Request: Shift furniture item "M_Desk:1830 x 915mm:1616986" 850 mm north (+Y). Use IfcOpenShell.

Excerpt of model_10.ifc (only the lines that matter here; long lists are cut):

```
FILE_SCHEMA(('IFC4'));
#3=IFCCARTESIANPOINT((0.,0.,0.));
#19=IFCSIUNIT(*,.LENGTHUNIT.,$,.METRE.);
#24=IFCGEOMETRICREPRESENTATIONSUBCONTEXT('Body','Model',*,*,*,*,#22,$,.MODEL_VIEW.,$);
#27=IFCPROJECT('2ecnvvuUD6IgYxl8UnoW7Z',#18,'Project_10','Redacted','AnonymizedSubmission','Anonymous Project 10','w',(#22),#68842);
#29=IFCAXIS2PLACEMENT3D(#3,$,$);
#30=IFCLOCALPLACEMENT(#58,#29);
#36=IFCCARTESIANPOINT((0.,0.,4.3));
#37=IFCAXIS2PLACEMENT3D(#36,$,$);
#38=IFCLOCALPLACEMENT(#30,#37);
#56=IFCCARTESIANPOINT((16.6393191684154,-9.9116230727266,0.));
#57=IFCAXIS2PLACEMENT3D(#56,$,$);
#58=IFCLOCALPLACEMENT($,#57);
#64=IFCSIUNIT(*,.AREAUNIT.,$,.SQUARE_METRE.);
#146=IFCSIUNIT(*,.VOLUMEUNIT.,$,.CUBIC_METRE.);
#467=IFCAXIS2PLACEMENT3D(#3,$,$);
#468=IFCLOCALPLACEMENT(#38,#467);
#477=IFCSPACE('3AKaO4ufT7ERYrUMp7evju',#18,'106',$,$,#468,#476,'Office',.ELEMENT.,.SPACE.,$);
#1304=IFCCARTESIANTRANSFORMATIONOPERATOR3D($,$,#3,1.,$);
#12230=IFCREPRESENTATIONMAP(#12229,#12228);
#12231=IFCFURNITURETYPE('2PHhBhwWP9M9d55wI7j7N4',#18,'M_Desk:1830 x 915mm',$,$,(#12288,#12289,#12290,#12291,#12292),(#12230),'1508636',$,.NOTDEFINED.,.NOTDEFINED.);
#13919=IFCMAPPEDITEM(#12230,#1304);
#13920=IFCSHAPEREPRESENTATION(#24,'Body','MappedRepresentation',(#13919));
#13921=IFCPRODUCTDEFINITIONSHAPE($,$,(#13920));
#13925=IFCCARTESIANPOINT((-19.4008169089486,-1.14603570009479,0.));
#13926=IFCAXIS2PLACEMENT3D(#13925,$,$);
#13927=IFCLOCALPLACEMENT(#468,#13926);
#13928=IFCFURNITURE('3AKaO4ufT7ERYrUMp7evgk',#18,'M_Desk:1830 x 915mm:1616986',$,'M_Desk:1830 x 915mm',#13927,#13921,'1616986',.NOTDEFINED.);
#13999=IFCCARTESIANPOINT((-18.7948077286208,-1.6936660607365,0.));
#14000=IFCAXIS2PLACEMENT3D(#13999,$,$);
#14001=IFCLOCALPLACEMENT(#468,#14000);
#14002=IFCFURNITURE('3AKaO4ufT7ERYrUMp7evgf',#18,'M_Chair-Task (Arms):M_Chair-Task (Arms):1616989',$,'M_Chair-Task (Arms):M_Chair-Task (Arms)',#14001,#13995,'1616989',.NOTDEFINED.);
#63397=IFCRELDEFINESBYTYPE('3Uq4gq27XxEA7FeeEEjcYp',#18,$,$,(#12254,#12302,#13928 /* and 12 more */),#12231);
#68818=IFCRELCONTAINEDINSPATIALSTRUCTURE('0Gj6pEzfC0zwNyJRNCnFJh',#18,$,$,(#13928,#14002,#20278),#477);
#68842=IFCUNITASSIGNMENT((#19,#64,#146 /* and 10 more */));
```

```python
import ifcopenshell
import ifcopenshell.api.geometry
import ifcopenshell.util.placement

model = ifcopenshell.open("model_10.ifc")

item = model.by_guid("3AKaO4ufT7ERYrUMp7evgk")
matrix = ifcopenshell.util.placement.get_local_placement(item.ObjectPlacement)
matrix[1, 3] += 0.85
ifcopenshell.api.geometry.edit_object_placement(model, product=item, matrix=matrix, is_si=False)

print(ifcopenshell.util.placement.get_local_placement(item.ObjectPlacement).round(3) + 0.0)

model.write("model_10_edited.ifc")
```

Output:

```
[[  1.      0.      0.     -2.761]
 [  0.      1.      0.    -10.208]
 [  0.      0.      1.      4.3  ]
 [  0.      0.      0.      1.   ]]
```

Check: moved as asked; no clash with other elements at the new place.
